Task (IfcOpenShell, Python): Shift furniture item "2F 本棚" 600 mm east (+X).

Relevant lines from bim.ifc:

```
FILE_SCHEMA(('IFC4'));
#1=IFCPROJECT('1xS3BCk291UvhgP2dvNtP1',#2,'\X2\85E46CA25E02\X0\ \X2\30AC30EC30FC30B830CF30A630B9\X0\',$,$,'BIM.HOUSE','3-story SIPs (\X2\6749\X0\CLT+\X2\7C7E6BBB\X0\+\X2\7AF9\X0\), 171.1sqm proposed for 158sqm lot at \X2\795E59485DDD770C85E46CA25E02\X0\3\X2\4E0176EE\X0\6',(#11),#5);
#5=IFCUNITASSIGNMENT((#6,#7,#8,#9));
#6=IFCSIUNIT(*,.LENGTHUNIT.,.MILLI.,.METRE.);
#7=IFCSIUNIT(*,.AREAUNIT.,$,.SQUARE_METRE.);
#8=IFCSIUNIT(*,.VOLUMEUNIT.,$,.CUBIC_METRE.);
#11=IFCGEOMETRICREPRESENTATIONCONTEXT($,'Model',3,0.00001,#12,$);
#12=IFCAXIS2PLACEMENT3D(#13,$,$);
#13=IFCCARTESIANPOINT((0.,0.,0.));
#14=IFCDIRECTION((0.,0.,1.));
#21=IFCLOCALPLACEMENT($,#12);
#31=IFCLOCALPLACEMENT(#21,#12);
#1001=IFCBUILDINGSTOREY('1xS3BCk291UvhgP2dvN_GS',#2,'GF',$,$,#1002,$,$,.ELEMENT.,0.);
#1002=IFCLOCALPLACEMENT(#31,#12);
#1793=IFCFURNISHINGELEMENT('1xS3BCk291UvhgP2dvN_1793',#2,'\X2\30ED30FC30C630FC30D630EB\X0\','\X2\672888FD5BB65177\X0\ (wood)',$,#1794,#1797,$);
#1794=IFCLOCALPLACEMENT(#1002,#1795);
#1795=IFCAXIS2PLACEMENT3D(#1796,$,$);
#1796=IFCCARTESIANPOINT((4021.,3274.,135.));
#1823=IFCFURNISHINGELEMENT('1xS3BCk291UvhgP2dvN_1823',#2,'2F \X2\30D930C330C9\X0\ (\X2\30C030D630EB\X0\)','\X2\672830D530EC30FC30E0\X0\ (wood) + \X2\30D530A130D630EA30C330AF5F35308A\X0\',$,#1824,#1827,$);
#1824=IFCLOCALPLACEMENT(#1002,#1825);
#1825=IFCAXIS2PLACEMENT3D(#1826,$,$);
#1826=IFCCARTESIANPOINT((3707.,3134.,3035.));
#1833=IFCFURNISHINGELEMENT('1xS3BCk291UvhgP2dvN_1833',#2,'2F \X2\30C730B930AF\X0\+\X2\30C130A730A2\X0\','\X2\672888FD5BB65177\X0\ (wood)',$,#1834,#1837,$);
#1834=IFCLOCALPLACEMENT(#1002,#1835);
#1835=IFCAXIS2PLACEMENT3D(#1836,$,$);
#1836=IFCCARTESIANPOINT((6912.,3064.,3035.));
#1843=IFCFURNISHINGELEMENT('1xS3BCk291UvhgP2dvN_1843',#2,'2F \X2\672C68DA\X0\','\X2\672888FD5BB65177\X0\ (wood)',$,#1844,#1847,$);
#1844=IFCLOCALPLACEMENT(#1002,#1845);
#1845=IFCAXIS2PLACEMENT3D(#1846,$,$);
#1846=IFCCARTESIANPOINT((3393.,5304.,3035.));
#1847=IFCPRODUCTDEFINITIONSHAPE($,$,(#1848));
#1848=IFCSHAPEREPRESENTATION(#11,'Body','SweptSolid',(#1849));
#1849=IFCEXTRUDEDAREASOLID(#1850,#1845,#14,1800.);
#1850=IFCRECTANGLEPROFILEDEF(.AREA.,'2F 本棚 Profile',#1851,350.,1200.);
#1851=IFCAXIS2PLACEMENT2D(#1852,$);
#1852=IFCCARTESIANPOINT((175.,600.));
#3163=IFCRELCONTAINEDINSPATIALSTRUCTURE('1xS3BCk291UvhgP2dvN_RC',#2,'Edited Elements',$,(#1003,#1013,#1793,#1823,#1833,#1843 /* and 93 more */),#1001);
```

```python
import ifcopenshell
import ifcopenshell.api.geometry
import ifcopenshell.util.placement

model = ifcopenshell.open("bim.ifc")

item = model.by_id(1843)
matrix = ifcopenshell.util.placement.get_local_placement(item.ObjectPlacement)
matrix[0, 3] += 600.0
ifcopenshell.api.geometry.edit_object_placement(model, product=item, matrix=matrix, is_si=False)

print(ifcopenshell.util.placement.get_local_placement(item.ObjectPlacement).round(3) + 0.0)

model.write("bim_rev.ifc")
```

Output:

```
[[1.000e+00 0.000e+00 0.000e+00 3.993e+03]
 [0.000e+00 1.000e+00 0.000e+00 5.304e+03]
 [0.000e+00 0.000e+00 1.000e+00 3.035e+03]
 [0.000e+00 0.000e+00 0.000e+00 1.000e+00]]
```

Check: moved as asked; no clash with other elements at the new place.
